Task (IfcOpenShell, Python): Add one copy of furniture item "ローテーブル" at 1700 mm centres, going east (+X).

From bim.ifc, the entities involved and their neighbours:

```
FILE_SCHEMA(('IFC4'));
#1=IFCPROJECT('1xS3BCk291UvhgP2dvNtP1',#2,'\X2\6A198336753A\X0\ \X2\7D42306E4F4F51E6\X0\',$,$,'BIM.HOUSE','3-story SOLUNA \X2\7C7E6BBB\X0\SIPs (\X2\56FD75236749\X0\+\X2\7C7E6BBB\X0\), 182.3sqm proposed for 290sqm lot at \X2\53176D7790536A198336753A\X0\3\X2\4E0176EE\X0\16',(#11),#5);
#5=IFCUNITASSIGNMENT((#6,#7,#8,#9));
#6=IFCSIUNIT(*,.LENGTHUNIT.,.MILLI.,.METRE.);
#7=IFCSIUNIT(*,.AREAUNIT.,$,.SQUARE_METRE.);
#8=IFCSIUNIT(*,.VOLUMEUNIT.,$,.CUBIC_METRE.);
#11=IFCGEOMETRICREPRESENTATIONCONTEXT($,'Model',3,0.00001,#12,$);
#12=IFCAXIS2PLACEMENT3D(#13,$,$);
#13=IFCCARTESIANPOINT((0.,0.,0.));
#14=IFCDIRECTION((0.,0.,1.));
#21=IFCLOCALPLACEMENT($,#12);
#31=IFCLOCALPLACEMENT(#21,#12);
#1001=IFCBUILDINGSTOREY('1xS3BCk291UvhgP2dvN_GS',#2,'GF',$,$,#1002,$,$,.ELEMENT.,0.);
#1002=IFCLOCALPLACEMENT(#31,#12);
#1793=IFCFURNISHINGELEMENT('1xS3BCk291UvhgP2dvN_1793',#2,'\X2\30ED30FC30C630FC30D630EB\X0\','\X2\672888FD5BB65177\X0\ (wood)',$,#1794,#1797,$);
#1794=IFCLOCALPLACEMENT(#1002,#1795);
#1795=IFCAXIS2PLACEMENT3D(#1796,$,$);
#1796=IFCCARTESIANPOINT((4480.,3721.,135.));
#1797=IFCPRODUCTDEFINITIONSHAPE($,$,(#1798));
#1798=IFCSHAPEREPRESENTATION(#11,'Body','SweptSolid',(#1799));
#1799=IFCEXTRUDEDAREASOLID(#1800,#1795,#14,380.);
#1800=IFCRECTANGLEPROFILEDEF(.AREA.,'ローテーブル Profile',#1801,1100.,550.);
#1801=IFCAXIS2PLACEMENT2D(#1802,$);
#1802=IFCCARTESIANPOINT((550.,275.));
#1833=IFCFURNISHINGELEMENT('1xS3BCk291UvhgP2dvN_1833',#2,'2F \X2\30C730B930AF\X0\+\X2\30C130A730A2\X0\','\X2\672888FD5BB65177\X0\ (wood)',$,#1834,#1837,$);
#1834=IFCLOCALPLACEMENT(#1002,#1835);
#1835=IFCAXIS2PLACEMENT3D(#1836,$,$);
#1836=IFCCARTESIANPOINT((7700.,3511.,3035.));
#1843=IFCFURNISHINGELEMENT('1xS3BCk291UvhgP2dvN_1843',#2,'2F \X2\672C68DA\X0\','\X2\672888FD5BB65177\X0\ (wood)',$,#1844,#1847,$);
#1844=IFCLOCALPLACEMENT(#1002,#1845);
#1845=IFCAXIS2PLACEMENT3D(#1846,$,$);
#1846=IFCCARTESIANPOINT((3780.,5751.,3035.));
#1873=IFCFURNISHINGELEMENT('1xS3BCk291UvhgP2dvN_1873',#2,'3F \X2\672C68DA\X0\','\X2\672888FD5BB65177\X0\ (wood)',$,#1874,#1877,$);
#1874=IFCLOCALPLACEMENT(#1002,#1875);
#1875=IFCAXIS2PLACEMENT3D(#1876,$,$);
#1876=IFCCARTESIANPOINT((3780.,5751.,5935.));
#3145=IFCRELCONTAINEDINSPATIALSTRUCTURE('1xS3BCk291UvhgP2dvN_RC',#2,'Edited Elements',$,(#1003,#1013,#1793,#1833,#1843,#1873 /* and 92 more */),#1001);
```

```python
import numpy as np
import ifcopenshell
import ifcopenshell.api.geometry
import ifcopenshell.api.root
import ifcopenshell.util.element
import ifcopenshell.util.placement

model = ifcopenshell.open("bim.ifc")


def reuse_history(source, copy):
    """copy_class also copies each property set's owner history, people and application; keep the originals."""
    for rel in copy.IsDefinedBy:
        if rel.is_a("IfcRelDefinesByProperties") and (history := rel.RelatingPropertyDefinition.OwnerHistory):
            rel.RelatingPropertyDefinition.OwnerHistory = source.OwnerHistory
            ifcopenshell.util.element.remove_deep2(model, history)


source = model.by_guid("1xS3BCk291UvhgP2dvN_1793")
base = ifcopenshell.util.placement.get_local_placement(source.ObjectPlacement)
step = np.array([1.0, 0.0, 0.0]) * 1700.0

for i in range(1, 2):
    copy = ifcopenshell.api.root.copy_class(model, product=source)
    copy.Representation = ifcopenshell.util.element.copy_deep(
        model, source.Representation, exclude=["IfcGeometricRepresentationContext", "IfcRepresentationMap"]
    )
    reuse_history(source, copy)
    matrix = base.copy()
    matrix[:3, 3] += i * step
    print("added at", matrix[:3, 3].round(3) + 0.0)
    ifcopenshell.api.geometry.edit_object_placement(model, product=copy, matrix=matrix, is_si=False)

model.write("bim_v2.ifc")
```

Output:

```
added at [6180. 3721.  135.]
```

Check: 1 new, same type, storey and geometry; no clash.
